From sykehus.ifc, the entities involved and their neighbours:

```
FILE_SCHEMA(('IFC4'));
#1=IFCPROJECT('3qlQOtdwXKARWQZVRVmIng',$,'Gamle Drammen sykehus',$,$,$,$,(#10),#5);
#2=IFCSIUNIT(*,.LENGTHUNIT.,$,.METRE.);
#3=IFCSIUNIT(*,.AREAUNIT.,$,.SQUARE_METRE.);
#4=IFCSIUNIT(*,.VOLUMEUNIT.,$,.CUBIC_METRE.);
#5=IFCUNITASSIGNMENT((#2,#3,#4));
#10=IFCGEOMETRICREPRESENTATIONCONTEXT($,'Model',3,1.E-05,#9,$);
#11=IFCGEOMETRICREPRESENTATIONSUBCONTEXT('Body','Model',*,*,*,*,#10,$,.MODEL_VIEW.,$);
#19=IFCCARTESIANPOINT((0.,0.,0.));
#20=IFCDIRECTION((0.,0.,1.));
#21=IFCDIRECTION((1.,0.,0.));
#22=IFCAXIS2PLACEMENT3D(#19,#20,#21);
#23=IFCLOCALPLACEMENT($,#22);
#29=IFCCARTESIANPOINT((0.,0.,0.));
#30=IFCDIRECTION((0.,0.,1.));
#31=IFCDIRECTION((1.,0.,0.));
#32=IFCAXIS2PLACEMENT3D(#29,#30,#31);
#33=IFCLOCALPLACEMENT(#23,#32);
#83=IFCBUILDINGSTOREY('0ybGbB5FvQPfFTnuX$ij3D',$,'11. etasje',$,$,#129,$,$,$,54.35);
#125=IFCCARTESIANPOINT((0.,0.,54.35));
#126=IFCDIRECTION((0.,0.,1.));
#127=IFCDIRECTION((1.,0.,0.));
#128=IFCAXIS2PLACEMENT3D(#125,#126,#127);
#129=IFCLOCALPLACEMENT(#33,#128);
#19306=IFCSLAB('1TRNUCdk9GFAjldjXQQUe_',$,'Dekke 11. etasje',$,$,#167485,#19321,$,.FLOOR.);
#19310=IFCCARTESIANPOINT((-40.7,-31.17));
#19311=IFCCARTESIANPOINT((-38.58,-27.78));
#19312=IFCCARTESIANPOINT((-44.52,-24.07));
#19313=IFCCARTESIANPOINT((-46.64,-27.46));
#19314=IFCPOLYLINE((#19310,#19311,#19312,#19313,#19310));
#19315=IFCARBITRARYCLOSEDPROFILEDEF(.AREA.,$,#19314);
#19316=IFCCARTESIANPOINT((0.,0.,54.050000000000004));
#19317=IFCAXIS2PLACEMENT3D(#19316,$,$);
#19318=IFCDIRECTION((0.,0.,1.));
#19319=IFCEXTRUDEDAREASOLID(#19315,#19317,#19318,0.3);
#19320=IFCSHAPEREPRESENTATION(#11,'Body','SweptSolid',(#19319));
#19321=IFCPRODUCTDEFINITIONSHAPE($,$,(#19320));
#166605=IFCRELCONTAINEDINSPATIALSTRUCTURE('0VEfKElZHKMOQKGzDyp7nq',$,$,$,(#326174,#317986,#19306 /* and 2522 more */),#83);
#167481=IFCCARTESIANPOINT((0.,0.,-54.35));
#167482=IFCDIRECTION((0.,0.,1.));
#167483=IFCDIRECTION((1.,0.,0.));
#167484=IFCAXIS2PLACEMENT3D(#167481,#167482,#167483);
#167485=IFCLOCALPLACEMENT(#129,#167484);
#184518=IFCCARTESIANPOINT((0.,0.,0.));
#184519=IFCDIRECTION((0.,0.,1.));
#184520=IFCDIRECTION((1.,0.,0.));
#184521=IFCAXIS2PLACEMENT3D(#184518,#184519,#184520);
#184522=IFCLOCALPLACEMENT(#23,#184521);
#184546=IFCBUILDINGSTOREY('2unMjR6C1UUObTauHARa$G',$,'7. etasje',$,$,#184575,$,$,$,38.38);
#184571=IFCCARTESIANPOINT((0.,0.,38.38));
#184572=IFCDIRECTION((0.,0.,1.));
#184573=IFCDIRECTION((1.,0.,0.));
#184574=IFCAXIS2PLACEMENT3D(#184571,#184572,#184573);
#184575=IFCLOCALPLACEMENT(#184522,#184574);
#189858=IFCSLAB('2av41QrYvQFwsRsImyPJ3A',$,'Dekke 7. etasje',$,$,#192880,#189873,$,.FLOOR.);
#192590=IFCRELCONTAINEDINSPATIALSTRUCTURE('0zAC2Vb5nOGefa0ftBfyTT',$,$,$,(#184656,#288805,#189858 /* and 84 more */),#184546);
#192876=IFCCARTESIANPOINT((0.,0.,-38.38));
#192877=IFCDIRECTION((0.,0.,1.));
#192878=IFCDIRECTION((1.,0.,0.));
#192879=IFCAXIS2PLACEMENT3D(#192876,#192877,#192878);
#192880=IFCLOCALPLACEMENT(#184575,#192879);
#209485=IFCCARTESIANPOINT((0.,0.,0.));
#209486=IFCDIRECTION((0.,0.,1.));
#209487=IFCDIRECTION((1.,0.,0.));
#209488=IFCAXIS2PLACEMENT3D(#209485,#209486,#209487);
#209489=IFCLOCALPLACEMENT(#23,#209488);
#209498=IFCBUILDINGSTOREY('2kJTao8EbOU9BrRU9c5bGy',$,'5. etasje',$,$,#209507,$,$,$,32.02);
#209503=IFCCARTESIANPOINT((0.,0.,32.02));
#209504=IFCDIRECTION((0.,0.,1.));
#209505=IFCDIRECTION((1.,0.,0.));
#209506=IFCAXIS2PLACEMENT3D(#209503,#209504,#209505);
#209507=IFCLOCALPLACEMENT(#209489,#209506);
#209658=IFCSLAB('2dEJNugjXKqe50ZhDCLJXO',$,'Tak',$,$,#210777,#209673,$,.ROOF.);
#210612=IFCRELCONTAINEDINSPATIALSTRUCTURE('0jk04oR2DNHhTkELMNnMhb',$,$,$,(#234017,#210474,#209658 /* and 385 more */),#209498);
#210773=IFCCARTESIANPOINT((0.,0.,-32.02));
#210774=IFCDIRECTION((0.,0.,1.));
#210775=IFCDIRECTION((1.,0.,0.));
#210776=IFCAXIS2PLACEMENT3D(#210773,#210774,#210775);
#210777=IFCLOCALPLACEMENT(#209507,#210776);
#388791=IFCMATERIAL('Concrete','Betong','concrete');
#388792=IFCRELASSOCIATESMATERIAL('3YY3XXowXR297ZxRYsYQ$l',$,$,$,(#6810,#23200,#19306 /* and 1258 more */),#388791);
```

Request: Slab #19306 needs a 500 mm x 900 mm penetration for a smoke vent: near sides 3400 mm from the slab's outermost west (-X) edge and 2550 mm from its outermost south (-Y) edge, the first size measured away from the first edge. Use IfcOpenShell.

```python
import numpy as np
import ifcopenshell
import ifcopenshell.api.feature
import ifcopenshell.api.geometry
import ifcopenshell.api.root
import ifcopenshell.geom
import ifcopenshell.util.placement
import ifcopenshell.util.representation
import ifcopenshell.util.shape
import ifcopenshell.util.unit

model = ifcopenshell.open("sykehus.ifc")
unit_scale = ifcopenshell.util.unit.calculate_unit_scale(model)
settings = ifcopenshell.geom.settings()


def volume(element):
    """Net volume in cubic metres, openings subtracted."""
    shape = ifcopenshell.geom.create_shape(settings, element)
    return ifcopenshell.util.shape.get_volume(shape.geometry)


slab = model.by_guid("1TRNUCdk9GFAjldjXQQUe_")
before = volume(slab)

# Extent in the slab's own axes, in metres. The edges named are its -X and -Y sides.
slab_shape = ifcopenshell.geom.create_shape(settings, slab)
vertices = ifcopenshell.util.shape.get_vertices(slab_shape.geometry)
x_min, y_min, bottom = vertices.min(axis=0)
top = vertices[:, 2].max()

opening = ifcopenshell.api.root.create_entity(model, ifc_class="IfcOpeningElement", name="Smoke vent opening", predefined_type="OPENING")
context = ifcopenshell.util.representation.get_context(model, "Model", "Body", "MODEL_VIEW")
width, depth = 0.5, 0.9
outline = [(0.0, 0.0), (width, 0.0), (width, depth), (0.0, depth), (0.0, 0.0)]
# Overshoot both faces by 50 mm so the cut is clean.
shape = ifcopenshell.api.geometry.add_slab_representation(
    model, context=context, depth=top - bottom + 0.1, polyline=outline
)
ifcopenshell.api.geometry.assign_representation(model, product=opening, representation=shape)

matrix = ifcopenshell.util.placement.get_local_placement(slab.ObjectPlacement)
matrix[:, 3] = matrix @ np.append(np.array([x_min + 3.4, y_min + 2.55, bottom - 0.05]) / unit_scale, 1.0)
ifcopenshell.api.geometry.edit_object_placement(model, product=opening, matrix=matrix, is_si=False)
ifcopenshell.api.feature.add_feature(model, feature=opening, element=slab)

after = volume(slab)

print(f"slab volume {before:.3f} -> {after:.3f} m3")

model.write("sykehus_edited.ifc")
```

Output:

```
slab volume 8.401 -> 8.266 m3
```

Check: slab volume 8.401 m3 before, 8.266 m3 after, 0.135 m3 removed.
